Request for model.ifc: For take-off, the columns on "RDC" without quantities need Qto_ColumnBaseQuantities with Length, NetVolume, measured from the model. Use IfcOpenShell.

First a look at what the model holds.

```python
import ifcopenshell
import ifcopenshell.util.element
import ifcopenshell.util.unit

model = ifcopenshell.open("model.ifc")
print(model.schema)
for unit_type in ("LENGTHUNIT", "AREAUNIT", "VOLUMEUNIT"):
    print(unit_type, ifcopenshell.util.unit.calculate_unit_scale(model, unit_type))
storey = next(s for s in model.by_type("IfcBuildingStorey") if s.Name == "RDC")
columns = [e for e in ifcopenshell.util.element.get_decomposition(storey) if e.is_a("IfcColumn")]
for e in sorted(columns, key=lambda e: e.id()):
    print(e.id(), e.is_a(), e.Name, list(ifcopenshell.util.element.get_psets(e, qtos_only=True)), sep=" | ")
```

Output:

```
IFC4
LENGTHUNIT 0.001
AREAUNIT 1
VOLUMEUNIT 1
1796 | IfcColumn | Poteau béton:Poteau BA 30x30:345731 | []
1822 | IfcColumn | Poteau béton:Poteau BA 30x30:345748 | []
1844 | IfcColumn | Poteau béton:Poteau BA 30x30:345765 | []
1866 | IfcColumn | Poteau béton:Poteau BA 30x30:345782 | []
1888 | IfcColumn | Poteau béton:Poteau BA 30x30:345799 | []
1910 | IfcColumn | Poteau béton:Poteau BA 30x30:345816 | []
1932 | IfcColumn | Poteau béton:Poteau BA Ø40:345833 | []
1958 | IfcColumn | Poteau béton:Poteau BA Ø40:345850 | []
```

```python
import ifcopenshell
import ifcopenshell.api.pset
import ifcopenshell.geom
import ifcopenshell.util.element
import ifcopenshell.util.shape
import ifcopenshell.util.unit

model = ifcopenshell.open("model.ifc")
unit_scale = ifcopenshell.util.unit.calculate_unit_scale(model)
volume_scale = ifcopenshell.util.unit.calculate_unit_scale(model, "VOLUMEUNIT")
settings = ifcopenshell.geom.settings()

storey = next(s for s in model.by_type("IfcBuildingStorey") if s.Name == "RDC")
columns = [e for e in ifcopenshell.util.element.get_decomposition(storey) if e.is_a("IfcColumn")]

for e in sorted(columns, key=lambda e: e.id()):
    if ifcopenshell.util.element.get_psets(e, qtos_only=True, should_inherit=False):
        continue
    # Geometry comes back in metres, in the element's own axes.
    shape = ifcopenshell.geom.create_shape(settings, e)
    values = {
        "Length": ifcopenshell.util.shape.get_z(shape.geometry) / unit_scale,
        "NetVolume": ifcopenshell.util.shape.get_volume(shape.geometry) / volume_scale,
    }
    qto = ifcopenshell.api.pset.add_qto(model, product=e, name="Qto_ColumnBaseQuantities")
    ifcopenshell.api.pset.edit_qto(model, qto=qto, properties=values)
    print(e.id(), {k: round(v, 3) for k, v in values.items()})

model.write("model_updated.ifc")
```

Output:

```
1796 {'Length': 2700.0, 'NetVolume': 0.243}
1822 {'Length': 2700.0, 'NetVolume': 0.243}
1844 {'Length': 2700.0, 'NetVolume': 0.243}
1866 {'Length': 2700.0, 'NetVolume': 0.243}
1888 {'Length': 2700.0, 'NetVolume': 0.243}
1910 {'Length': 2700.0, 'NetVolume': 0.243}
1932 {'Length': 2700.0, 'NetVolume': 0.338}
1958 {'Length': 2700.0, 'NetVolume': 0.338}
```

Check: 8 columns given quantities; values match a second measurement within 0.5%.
